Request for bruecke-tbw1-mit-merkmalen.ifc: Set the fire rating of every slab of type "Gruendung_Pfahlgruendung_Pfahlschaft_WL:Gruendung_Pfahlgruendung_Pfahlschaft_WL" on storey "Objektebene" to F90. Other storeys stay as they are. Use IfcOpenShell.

First a look at what the model holds.

```python
import ifcopenshell
import ifcopenshell.util.element

model = ifcopenshell.open("bruecke-tbw1-mit-merkmalen.ifc")
print(model.schema)
storey = next(s for s in model.by_type("IfcBuildingStorey") if s.Name == "Objektebene")
slabs = [e for e in ifcopenshell.util.element.get_decomposition(storey) if e.is_a("IfcSlab")]
seen = {}
for e in slabs:
    element_type = ifcopenshell.util.element.get_type(e)
    key = (element_type.Name if element_type != e and element_type else None, ifcopenshell.util.element.get_pset(e, "Pset_SlabCommon", "FireRating"))
    seen[key] = seen.get(key, 0) + 1
for (name, value), count in sorted(seen.items(), key=str):
    print(count, "x", name, "|", value)
```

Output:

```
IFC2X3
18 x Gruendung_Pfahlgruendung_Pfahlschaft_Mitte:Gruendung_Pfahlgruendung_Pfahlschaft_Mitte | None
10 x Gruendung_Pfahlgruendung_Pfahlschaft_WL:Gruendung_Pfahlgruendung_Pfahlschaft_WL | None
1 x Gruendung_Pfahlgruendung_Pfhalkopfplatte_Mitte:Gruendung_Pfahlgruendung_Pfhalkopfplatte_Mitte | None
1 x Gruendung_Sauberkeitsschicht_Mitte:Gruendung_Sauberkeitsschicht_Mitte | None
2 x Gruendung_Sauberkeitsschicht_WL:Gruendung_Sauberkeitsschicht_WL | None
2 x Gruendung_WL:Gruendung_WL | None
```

```python
import ifcopenshell
import ifcopenshell.api.pset
import ifcopenshell.util.element

model = ifcopenshell.open("bruecke-tbw1-mit-merkmalen.ifc")

storey = next(s for s in model.by_type("IfcBuildingStorey") if s.Name == "Objektebene")
slabs = [e for e in ifcopenshell.util.element.get_decomposition(storey) if e.is_a("IfcSlab")]

count = 0
for e in slabs:
    element_type = ifcopenshell.util.element.get_type(e)
    if element_type in (None, e) or element_type.Name != "Gruendung_Pfahlgruendung_Pfahlschaft_WL:Gruendung_Pfahlgruendung_Pfahlschaft_WL":
        continue
    # add_pset returns the element's existing set when there is one.
    pset = ifcopenshell.api.pset.add_pset(model, product=e, name="Pset_SlabCommon")
    ifcopenshell.api.pset.edit_pset(model, pset=pset, properties={"FireRating": "F90"})
    count += 1

print(count, "slabs updated")

model.write("bruecke-tbw1-mit-merkmalen_updated.ifc")
```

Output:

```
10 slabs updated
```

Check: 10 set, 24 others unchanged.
